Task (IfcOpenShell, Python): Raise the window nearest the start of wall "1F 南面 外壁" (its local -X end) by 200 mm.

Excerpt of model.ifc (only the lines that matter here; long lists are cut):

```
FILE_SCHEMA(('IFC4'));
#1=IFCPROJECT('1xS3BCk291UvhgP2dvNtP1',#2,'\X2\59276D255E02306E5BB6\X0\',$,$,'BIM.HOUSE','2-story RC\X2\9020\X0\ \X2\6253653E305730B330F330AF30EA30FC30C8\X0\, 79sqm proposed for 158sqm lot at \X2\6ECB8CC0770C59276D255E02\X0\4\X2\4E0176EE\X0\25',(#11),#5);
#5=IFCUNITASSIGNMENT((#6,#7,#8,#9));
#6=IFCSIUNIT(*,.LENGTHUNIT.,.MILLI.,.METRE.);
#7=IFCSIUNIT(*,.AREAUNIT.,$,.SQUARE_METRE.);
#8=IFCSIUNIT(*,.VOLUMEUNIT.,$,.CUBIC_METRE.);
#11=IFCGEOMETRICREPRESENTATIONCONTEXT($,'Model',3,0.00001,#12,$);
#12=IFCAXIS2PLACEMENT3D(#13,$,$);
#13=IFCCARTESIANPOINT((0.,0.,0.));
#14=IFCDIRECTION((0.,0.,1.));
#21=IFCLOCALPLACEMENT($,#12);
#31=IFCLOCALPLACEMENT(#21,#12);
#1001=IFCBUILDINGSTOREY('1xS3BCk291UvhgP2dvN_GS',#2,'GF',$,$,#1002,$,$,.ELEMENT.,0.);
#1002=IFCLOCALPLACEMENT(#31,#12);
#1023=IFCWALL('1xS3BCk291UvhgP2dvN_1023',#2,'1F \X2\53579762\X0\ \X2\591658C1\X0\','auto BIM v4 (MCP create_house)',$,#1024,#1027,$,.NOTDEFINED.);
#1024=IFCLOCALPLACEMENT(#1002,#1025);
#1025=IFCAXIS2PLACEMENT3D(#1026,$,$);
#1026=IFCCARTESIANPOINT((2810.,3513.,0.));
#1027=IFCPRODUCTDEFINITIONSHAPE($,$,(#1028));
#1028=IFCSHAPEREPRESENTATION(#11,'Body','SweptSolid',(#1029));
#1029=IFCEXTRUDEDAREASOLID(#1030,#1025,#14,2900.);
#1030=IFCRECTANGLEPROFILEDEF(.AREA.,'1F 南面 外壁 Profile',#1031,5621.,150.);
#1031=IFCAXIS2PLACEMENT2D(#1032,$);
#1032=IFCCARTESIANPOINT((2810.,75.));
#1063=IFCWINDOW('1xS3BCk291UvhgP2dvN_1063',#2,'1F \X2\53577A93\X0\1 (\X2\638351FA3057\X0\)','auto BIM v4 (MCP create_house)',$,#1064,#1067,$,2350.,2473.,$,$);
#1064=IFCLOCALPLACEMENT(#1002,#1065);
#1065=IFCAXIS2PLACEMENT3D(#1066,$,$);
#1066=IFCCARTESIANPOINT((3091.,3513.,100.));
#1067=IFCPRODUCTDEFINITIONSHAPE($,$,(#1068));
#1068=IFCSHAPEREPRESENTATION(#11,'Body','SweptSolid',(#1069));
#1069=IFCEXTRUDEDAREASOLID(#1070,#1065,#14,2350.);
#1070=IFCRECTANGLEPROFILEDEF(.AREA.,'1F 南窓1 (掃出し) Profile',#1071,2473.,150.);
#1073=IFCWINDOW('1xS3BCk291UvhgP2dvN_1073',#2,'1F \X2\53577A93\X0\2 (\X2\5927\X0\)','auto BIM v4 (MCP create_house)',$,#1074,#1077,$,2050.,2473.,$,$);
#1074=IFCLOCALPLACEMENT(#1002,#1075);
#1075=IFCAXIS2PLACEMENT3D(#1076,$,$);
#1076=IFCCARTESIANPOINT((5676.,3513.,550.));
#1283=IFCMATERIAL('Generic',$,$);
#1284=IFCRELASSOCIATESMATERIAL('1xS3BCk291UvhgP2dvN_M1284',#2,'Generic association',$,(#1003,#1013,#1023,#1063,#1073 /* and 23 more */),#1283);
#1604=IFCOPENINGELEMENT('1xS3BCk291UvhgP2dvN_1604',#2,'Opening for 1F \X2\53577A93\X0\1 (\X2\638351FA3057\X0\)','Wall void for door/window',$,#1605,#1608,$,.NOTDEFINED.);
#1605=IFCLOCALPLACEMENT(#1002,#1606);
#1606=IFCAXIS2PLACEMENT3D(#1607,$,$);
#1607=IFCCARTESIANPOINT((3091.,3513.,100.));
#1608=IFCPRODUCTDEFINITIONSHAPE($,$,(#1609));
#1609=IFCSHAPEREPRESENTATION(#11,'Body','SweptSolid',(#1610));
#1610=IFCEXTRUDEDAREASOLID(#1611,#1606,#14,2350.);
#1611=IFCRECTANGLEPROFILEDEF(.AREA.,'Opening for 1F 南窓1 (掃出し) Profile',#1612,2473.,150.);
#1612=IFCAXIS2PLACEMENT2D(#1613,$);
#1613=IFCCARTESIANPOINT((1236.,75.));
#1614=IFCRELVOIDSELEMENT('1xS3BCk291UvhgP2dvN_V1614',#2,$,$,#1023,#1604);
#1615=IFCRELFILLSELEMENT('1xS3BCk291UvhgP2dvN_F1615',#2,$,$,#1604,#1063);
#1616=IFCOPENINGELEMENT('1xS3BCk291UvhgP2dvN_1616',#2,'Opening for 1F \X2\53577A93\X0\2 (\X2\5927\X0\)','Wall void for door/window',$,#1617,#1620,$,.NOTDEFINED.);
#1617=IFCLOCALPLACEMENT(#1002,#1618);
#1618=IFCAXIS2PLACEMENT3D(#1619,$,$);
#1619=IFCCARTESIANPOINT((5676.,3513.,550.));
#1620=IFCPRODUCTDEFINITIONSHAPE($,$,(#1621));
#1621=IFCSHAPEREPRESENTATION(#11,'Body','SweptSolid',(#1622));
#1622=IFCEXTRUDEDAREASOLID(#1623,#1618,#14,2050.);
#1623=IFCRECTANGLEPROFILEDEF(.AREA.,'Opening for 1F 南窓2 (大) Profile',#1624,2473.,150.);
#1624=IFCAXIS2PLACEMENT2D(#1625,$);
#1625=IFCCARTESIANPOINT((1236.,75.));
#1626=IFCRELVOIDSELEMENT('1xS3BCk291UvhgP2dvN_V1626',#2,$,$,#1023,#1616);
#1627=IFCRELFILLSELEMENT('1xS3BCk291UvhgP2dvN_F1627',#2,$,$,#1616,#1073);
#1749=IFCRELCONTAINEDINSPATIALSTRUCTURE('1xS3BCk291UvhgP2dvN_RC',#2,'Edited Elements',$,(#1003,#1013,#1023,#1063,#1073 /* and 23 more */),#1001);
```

```python
import numpy as np
import ifcopenshell
import ifcopenshell.api.geometry
import ifcopenshell.util.placement
import ifcopenshell.util.unit

model = ifcopenshell.open("model.ifc")
unit_scale = ifcopenshell.util.unit.calculate_unit_scale(model)

window = model.by_guid("1xS3BCk291UvhgP2dvN_1063")
opening = window.FillsVoids[0].RelatingOpeningElement
dz = 200.0

shift = np.array([0.0, 0.0, dz])
# The window is not placed relative to its opening, so move both.
for product in (opening, window):
    matrix = ifcopenshell.util.placement.get_local_placement(product.ObjectPlacement)
    matrix[:3, 3] += shift
    ifcopenshell.api.geometry.edit_object_placement(model, product=product, matrix=matrix, is_si=False)

print(f"moved by {dz * unit_scale:+.3f} m")

model.write("model_v2.ifc")
```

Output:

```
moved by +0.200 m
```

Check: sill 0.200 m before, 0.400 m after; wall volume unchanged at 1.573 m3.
